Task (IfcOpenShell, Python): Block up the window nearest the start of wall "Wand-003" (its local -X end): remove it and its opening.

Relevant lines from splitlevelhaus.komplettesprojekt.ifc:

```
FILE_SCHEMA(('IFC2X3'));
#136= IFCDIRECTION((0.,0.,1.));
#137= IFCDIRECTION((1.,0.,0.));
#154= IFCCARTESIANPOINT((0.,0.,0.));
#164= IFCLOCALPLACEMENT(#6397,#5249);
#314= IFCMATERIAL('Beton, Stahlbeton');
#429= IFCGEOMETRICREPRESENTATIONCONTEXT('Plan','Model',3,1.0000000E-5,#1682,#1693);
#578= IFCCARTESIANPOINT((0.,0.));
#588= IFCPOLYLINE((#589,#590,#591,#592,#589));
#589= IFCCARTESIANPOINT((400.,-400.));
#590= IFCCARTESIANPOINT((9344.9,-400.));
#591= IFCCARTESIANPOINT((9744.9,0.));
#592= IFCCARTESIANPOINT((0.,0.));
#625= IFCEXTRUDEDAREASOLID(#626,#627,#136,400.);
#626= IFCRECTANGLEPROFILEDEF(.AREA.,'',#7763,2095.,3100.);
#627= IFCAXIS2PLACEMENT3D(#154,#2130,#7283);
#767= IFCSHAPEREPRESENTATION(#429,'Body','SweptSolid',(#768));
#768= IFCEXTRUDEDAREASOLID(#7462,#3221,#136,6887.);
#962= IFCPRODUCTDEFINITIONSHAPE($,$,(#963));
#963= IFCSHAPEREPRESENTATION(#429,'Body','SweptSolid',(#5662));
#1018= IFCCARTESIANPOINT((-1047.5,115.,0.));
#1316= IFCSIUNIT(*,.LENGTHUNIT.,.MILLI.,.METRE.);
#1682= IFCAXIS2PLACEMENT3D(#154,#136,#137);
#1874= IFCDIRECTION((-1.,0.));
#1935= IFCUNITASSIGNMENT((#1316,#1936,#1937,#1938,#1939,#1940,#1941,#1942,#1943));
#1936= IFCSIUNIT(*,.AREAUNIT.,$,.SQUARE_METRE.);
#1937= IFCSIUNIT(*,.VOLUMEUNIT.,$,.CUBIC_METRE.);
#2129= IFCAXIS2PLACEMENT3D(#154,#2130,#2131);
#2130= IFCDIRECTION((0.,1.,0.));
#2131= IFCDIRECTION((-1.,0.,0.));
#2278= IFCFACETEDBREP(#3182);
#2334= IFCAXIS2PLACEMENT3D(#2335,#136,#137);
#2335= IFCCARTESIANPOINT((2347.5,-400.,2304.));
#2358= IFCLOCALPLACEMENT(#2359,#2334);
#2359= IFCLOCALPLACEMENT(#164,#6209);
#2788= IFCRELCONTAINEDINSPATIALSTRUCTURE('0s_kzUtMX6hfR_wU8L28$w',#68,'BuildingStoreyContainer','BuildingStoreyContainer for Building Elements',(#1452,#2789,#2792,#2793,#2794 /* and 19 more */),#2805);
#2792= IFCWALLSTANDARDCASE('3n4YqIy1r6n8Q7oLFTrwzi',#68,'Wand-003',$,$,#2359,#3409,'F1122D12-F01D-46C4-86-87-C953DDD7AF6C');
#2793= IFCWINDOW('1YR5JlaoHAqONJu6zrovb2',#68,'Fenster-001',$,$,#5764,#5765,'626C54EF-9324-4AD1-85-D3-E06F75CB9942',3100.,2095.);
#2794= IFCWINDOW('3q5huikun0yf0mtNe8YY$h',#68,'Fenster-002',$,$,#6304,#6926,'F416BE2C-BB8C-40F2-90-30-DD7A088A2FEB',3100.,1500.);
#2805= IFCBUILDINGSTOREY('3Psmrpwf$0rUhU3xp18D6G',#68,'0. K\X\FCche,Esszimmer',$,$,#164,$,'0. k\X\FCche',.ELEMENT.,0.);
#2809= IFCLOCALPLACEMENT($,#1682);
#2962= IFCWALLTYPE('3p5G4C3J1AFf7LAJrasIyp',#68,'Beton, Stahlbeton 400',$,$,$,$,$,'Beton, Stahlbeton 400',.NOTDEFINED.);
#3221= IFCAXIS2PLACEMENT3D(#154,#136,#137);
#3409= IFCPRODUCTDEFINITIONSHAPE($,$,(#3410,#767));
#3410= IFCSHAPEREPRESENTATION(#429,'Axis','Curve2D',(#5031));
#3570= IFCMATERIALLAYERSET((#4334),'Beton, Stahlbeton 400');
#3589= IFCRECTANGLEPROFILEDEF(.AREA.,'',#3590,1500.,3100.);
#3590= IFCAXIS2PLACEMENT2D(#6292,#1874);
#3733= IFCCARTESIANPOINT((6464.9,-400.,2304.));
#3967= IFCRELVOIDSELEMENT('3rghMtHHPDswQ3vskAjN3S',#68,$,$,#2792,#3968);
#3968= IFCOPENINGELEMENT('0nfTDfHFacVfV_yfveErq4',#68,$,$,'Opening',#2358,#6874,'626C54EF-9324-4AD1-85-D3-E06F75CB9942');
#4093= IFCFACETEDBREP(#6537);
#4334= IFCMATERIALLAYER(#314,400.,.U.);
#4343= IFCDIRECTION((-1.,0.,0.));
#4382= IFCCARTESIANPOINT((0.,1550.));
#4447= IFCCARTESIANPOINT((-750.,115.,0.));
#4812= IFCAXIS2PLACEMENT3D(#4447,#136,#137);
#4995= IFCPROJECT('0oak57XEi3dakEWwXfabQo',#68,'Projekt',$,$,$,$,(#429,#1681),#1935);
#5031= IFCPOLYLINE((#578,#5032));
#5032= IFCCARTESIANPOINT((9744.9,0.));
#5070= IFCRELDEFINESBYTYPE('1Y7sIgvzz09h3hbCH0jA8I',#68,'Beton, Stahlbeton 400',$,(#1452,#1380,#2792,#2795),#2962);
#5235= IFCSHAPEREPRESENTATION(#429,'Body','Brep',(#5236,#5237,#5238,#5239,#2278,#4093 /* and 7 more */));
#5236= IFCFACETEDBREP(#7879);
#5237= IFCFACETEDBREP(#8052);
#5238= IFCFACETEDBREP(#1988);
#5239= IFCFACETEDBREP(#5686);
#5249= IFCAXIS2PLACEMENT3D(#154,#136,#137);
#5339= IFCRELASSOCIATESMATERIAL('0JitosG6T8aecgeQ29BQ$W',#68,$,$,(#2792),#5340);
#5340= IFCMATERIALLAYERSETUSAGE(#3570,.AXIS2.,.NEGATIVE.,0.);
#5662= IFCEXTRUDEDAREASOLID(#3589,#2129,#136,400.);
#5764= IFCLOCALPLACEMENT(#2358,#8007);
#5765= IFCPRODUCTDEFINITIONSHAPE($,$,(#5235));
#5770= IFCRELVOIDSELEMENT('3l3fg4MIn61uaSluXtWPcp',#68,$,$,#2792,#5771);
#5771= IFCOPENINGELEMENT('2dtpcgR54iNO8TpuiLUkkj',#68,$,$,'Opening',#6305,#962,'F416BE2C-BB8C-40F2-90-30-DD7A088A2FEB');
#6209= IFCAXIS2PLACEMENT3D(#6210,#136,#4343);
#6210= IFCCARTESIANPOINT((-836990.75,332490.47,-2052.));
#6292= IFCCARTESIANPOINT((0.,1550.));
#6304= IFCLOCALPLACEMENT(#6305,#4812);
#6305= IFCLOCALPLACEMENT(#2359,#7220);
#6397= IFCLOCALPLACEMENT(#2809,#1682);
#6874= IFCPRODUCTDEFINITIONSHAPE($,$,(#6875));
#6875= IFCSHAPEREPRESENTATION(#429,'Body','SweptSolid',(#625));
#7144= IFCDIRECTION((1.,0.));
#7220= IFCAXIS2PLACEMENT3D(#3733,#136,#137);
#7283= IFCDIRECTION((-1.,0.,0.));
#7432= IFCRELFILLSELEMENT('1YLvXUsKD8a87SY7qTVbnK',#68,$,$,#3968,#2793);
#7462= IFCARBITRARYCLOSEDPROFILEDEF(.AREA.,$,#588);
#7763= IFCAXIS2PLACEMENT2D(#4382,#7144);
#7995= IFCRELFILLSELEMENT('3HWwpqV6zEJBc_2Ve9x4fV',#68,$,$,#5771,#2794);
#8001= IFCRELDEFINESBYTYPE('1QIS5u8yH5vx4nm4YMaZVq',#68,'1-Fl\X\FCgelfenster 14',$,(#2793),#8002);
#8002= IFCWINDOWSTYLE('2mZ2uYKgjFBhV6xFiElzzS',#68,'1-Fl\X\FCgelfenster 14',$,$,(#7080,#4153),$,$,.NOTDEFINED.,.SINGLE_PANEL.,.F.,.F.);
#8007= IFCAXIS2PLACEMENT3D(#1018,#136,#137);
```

```python
import ifcopenshell
import ifcopenshell.api.feature
import ifcopenshell.api.root
import ifcopenshell.geom
import ifcopenshell.util.shape

model = ifcopenshell.open("splitlevelhaus.komplettesprojekt.ifc")
settings = ifcopenshell.geom.settings()


def volume(element):
    """Net volume in cubic metres, openings subtracted."""
    shape = ifcopenshell.geom.create_shape(settings, element)
    return ifcopenshell.util.shape.get_volume(shape.geometry)


window = model.by_guid("1YR5JlaoHAqONJu6zrovb2")
opening = window.FillsVoids[0].RelatingOpeningElement
wall = opening.VoidsElements[0].RelatingBuildingElement
before = volume(wall)

ifcopenshell.api.root.remove_product(model, product=window)
ifcopenshell.api.feature.remove_feature(model, feature=opening)

after = volume(wall)

print(f"wall volume {before:.3f} -> {after:.3f} m3")

model.write("splitlevelhaus.komplettesprojekt_v2.ifc")
```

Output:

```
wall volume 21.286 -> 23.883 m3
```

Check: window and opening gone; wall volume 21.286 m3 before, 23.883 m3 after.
